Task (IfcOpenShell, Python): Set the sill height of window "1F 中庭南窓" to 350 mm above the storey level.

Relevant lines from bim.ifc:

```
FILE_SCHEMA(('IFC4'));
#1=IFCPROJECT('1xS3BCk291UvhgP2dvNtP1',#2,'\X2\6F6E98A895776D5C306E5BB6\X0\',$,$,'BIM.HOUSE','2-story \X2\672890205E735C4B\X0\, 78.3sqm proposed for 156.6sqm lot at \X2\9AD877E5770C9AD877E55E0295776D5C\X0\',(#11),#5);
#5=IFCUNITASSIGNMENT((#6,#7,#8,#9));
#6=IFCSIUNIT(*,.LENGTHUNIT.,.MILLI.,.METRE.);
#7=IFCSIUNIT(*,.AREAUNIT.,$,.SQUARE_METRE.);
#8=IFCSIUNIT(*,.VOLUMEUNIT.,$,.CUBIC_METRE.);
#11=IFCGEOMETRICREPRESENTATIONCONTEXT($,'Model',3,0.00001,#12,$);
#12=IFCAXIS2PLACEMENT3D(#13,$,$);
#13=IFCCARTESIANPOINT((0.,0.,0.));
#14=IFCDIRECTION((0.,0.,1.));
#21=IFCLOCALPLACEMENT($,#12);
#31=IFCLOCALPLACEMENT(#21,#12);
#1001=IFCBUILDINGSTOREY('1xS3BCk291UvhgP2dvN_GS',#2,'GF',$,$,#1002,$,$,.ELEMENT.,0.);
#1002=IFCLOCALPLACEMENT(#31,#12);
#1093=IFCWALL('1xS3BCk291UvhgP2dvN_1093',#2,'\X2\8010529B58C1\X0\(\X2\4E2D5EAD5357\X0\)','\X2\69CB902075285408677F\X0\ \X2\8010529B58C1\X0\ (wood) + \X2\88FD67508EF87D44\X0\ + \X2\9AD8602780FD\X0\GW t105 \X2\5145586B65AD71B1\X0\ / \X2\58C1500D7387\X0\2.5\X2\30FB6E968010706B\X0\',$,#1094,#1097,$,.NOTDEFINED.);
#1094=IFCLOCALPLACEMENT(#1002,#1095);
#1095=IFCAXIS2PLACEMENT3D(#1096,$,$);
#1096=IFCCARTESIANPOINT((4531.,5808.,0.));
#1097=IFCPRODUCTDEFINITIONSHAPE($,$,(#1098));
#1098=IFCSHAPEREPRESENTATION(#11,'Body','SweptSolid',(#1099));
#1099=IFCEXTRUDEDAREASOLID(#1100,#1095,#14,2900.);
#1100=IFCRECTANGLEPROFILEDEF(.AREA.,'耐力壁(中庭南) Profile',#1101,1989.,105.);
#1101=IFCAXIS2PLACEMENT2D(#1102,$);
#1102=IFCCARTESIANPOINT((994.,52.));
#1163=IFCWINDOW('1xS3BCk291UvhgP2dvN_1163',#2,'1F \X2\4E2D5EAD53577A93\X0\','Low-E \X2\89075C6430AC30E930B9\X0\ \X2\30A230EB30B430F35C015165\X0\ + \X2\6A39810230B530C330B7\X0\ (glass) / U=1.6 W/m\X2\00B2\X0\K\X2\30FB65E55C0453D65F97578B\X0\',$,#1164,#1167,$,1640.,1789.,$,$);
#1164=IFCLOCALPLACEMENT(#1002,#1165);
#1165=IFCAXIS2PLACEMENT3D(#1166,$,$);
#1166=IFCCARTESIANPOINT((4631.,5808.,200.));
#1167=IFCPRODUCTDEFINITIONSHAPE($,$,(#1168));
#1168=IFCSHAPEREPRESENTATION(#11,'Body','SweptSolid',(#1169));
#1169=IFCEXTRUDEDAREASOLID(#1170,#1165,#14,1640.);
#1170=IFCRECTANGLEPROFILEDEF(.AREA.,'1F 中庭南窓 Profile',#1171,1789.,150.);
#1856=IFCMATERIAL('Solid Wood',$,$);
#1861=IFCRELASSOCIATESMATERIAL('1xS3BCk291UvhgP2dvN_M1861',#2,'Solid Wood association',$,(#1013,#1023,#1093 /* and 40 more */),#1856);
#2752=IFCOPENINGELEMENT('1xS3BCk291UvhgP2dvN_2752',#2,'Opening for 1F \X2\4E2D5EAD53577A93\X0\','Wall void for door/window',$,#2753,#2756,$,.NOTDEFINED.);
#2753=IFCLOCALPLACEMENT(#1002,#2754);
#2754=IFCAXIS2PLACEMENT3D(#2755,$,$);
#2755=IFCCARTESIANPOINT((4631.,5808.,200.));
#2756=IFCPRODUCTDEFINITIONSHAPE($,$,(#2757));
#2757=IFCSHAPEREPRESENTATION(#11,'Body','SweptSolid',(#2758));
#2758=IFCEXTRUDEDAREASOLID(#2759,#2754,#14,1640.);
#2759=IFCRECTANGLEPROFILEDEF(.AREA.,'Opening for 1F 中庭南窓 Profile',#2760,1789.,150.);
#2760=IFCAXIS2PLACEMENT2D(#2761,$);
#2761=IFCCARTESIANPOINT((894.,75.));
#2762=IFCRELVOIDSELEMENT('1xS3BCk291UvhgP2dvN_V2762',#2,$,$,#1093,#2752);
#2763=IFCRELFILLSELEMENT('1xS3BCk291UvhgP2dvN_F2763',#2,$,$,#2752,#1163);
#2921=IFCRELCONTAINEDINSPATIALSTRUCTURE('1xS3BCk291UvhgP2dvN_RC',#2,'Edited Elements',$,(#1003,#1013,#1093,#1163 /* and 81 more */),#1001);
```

```python
import numpy as np
import ifcopenshell
import ifcopenshell.api.geometry
import ifcopenshell.geom
import ifcopenshell.util.element
import ifcopenshell.util.placement
import ifcopenshell.util.shape
import ifcopenshell.util.unit

model = ifcopenshell.open("bim.ifc")
unit_scale = ifcopenshell.util.unit.calculate_unit_scale(model)

window = model.by_id(1163)
opening = window.FillsVoids[0].RelatingOpeningElement
storey = ifcopenshell.util.element.get_container(window, ifc_class="IfcBuildingStorey")
level = ifcopenshell.util.placement.get_local_placement(storey.ObjectPlacement)[2, 3]

# The opening's origin need not be at the sill, so measure its lowest point.
shape = ifcopenshell.geom.create_shape(ifcopenshell.geom.settings(), opening)
bottom = ifcopenshell.util.shape.get_shape_bottom_elevation(shape, shape.geometry) / unit_scale
dz = level + 0.35 / unit_scale - bottom

shift = np.array([0.0, 0.0, dz])
# The window is not placed relative to its opening, so move both.
for product in (opening, window):
    matrix = ifcopenshell.util.placement.get_local_placement(product.ObjectPlacement)
    matrix[:3, 3] += shift
    ifcopenshell.api.geometry.edit_object_placement(model, product=product, matrix=matrix, is_si=False)

print(f"moved by {dz * unit_scale:+.3f} m")

model.write("bim_rev.ifc")
```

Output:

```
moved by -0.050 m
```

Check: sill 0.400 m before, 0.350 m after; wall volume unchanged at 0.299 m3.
